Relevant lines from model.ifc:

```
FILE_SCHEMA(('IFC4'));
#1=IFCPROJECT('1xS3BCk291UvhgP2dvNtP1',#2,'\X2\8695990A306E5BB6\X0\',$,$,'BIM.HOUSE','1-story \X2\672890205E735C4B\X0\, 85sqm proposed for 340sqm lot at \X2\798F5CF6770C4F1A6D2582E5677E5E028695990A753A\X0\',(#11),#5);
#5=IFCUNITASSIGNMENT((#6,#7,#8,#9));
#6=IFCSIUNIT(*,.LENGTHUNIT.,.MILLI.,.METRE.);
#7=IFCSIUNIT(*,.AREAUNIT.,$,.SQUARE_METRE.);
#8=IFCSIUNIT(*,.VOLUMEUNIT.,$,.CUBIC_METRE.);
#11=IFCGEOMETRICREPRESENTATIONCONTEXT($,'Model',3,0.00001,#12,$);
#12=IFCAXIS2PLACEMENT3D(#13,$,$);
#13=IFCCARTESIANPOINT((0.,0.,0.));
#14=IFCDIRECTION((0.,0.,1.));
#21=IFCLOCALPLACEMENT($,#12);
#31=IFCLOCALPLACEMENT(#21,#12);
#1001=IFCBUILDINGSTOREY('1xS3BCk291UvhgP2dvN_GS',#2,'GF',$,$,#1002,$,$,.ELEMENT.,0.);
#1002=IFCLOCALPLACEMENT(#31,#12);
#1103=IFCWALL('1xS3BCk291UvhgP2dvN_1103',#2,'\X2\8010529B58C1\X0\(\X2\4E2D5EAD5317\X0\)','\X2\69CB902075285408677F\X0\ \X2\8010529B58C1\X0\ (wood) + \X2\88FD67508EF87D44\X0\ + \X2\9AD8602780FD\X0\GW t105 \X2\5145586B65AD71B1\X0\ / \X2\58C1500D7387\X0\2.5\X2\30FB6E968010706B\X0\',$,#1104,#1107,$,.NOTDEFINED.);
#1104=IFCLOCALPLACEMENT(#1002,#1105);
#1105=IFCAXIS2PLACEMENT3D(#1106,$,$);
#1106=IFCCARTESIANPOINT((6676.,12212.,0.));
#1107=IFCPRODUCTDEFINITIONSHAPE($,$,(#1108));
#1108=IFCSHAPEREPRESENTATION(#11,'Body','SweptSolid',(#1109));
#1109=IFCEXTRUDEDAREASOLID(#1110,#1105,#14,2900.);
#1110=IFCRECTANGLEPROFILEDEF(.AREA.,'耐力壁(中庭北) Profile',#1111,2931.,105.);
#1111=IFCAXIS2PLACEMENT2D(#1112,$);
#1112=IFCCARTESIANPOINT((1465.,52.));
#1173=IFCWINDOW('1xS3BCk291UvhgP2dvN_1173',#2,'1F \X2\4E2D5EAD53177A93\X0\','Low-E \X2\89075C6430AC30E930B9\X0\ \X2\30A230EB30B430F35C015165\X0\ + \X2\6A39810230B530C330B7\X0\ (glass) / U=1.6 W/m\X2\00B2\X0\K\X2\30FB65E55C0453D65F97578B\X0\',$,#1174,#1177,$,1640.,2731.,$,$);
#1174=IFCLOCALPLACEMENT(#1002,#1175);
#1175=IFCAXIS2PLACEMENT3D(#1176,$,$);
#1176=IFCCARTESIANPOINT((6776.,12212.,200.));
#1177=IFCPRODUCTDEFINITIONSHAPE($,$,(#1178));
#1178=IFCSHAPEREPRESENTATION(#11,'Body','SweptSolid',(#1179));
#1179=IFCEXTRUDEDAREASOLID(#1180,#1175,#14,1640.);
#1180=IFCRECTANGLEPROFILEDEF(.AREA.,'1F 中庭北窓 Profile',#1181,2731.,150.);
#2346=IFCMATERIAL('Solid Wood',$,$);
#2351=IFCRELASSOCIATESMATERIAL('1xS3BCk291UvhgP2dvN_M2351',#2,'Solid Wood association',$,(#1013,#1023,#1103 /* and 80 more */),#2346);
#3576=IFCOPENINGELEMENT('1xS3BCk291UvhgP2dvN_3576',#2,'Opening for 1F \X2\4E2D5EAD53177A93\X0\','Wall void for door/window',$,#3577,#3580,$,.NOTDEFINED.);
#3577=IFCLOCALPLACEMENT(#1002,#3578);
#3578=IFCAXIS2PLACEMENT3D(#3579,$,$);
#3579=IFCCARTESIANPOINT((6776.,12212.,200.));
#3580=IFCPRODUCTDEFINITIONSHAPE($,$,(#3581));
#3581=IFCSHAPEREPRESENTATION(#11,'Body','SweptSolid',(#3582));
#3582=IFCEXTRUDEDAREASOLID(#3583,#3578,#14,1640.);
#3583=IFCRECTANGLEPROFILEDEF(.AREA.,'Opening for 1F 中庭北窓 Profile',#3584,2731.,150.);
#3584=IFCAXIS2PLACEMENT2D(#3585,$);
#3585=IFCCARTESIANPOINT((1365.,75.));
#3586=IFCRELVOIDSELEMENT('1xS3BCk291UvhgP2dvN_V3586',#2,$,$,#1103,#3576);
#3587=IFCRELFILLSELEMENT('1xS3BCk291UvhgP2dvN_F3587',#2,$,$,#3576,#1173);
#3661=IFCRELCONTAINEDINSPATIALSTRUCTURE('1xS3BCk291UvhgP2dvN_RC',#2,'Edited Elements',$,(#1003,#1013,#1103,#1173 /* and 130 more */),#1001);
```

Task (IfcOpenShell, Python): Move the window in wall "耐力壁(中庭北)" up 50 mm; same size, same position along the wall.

```python
import numpy as np
import ifcopenshell
import ifcopenshell.api.geometry
import ifcopenshell.util.placement
import ifcopenshell.util.unit

model = ifcopenshell.open("model.ifc")
unit_scale = ifcopenshell.util.unit.calculate_unit_scale(model)

window = model.by_guid("1xS3BCk291UvhgP2dvN_1173")
opening = window.FillsVoids[0].RelatingOpeningElement
dz = 0.05 / unit_scale

shift = np.array([0.0, 0.0, dz])
# The window is not placed relative to its opening, so move both.
for product in (opening, window):
    matrix = ifcopenshell.util.placement.get_local_placement(product.ObjectPlacement)
    matrix[:3, 3] += shift
    ifcopenshell.api.geometry.edit_object_placement(model, product=product, matrix=matrix, is_si=False)

print(f"moved by {dz * unit_scale:+.3f} m")

model.write("model_rev.ifc")
```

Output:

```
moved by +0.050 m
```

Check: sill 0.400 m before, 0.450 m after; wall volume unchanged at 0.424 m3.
